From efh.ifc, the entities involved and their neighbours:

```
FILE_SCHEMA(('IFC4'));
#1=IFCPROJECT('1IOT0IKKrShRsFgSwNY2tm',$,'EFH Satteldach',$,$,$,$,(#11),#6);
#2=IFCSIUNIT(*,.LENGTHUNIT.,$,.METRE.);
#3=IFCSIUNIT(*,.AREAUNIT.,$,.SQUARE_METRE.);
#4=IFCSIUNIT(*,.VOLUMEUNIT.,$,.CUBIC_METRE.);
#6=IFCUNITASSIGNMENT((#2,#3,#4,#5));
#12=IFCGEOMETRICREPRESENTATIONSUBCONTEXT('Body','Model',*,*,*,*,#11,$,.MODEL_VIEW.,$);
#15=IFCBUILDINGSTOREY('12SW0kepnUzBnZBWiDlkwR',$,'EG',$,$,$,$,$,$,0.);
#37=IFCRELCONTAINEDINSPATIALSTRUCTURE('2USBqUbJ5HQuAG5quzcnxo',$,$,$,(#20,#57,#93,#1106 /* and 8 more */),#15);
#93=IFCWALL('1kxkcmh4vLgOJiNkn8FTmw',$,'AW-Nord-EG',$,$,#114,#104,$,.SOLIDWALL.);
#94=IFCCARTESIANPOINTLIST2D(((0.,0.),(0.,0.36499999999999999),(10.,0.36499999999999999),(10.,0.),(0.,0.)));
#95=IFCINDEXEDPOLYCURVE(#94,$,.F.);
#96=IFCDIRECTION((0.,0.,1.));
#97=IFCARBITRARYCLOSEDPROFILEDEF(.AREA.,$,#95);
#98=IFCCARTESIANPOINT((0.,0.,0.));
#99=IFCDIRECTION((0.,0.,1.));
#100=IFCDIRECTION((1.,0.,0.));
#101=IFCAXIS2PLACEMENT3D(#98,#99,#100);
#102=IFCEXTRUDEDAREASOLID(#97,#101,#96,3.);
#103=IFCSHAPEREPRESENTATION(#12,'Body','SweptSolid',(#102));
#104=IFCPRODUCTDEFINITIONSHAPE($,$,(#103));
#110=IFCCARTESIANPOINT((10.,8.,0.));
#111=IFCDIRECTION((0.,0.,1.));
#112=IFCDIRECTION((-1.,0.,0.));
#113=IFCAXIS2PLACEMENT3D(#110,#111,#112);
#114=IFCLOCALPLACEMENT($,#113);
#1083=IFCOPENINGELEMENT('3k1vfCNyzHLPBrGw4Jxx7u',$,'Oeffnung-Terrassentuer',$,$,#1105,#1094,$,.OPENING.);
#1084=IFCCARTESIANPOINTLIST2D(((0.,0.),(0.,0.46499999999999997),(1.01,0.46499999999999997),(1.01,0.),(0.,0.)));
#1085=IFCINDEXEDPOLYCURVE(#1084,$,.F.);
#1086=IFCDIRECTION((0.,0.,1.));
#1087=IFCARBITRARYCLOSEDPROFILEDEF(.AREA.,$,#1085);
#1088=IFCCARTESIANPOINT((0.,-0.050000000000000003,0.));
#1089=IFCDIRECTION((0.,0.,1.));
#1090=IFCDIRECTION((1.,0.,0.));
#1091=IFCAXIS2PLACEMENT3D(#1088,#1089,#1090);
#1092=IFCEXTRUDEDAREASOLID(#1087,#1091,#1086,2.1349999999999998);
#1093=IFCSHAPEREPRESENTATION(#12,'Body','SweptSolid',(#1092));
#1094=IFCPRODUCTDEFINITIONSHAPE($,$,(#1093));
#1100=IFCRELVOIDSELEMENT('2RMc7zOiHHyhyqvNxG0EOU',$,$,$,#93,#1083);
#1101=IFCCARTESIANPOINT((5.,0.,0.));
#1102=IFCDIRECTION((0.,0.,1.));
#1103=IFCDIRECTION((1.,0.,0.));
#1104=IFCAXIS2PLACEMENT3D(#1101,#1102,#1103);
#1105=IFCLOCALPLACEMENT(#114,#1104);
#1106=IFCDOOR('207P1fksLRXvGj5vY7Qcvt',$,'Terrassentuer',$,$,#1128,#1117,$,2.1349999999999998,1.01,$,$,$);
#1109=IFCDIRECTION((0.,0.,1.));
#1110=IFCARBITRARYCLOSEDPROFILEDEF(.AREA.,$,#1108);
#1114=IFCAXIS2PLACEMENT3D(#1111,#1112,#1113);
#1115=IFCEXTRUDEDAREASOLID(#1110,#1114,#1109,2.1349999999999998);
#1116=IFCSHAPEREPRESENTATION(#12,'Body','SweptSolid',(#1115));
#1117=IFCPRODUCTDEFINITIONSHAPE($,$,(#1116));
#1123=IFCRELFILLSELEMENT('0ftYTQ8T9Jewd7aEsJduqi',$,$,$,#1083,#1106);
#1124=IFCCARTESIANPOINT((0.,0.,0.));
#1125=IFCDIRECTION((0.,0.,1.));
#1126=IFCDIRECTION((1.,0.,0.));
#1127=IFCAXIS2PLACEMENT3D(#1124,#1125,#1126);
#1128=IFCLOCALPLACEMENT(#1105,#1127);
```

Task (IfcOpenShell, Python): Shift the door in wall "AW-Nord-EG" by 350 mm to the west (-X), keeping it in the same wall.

```python
import ifcopenshell
import ifcopenshell.api.geometry
import ifcopenshell.util.placement
import ifcopenshell.util.unit

model = ifcopenshell.open("efh.ifc")
unit_scale = ifcopenshell.util.unit.calculate_unit_scale(model)

door = model.by_guid("207P1fksLRXvGj5vY7Qcvt")
opening = door.FillsVoids[0].RelatingOpeningElement
wall = opening.VoidsElements[0].RelatingBuildingElement

wall_matrix = ifcopenshell.util.placement.get_local_placement(wall.ObjectPlacement)
shift = wall_matrix[:3, 0] * 0.35 / unit_scale
before = ifcopenshell.util.placement.get_local_placement(door.ObjectPlacement)[:3, 3].copy()

# The door is placed relative to its opening, so it follows when the opening moves.
matrix = ifcopenshell.util.placement.get_local_placement(opening.ObjectPlacement)
matrix[:3, 3] += shift
ifcopenshell.api.geometry.edit_object_placement(
    model, product=opening, matrix=matrix, is_si=False, should_transform_children=True
)

after = ifcopenshell.util.placement.get_local_placement(door.ObjectPlacement)[:3, 3]
print("door moved by", (after - before).round(3) + 0.0)

model.write("efh-out.ifc")
```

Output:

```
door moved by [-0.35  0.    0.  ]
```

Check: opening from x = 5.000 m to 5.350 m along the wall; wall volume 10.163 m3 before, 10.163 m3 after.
